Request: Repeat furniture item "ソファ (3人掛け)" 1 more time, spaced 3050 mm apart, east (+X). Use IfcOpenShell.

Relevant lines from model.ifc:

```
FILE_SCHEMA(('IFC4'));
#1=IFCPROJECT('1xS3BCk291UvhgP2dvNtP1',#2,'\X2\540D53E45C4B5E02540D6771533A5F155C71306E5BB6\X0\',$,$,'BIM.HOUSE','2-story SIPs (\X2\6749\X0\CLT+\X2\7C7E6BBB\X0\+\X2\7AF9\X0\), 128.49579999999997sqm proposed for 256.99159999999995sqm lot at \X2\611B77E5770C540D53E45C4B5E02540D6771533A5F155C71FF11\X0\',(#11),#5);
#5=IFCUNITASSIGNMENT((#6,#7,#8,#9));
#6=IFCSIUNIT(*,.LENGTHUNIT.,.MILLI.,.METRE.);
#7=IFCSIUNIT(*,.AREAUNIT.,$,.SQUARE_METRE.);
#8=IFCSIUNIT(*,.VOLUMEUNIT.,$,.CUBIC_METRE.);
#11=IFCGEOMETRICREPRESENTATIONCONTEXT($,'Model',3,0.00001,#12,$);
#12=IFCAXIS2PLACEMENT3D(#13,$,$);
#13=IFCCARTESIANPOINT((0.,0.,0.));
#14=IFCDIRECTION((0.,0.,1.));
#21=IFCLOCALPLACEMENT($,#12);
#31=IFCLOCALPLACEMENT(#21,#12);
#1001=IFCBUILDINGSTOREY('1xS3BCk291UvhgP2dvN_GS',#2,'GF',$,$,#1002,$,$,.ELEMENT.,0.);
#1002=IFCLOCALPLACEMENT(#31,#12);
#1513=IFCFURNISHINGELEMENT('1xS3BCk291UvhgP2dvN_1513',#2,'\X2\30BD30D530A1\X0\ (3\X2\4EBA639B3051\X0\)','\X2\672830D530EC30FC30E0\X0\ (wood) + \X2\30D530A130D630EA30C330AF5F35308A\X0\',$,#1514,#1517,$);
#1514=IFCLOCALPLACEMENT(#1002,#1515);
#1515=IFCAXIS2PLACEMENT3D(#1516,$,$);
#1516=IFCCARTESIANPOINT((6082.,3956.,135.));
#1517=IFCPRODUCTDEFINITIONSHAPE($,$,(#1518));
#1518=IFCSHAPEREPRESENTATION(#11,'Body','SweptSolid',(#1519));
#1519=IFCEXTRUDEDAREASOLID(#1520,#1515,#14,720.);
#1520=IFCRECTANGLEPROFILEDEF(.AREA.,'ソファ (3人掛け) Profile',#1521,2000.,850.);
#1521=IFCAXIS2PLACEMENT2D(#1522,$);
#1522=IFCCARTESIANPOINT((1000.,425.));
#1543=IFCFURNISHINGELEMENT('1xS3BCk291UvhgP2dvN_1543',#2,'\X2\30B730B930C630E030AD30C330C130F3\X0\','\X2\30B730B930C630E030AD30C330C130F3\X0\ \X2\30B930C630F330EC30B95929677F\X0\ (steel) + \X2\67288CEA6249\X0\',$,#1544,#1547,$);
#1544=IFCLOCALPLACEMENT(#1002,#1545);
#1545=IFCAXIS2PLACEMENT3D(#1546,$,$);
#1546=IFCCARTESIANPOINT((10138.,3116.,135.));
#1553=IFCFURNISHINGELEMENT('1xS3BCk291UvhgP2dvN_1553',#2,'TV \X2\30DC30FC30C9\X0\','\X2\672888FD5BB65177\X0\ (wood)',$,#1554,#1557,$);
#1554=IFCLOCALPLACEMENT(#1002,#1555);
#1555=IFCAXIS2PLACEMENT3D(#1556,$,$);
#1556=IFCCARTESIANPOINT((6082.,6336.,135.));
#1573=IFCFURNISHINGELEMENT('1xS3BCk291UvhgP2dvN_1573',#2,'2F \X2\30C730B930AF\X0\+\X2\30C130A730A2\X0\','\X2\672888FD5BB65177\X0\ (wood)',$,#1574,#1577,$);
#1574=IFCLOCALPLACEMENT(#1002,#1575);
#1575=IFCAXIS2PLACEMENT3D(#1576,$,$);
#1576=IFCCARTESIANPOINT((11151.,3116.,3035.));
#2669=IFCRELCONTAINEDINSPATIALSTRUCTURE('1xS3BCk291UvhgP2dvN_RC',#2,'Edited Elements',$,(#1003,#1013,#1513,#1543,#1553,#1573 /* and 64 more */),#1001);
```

```python
import numpy as np
import ifcopenshell
import ifcopenshell.api.geometry
import ifcopenshell.api.root
import ifcopenshell.util.element
import ifcopenshell.util.placement

model = ifcopenshell.open("model.ifc")


def reuse_history(source, copy):
    """copy_class also copies each property set's owner history, people and application; keep the originals."""
    for rel in copy.IsDefinedBy:
        if rel.is_a("IfcRelDefinesByProperties") and (history := rel.RelatingPropertyDefinition.OwnerHistory):
            rel.RelatingPropertyDefinition.OwnerHistory = source.OwnerHistory
            ifcopenshell.util.element.remove_deep2(model, history)


source = model.by_guid("1xS3BCk291UvhgP2dvN_1513")
base = ifcopenshell.util.placement.get_local_placement(source.ObjectPlacement)
step = np.array([1.0, 0.0, 0.0]) * 3050.0

for i in range(1, 2):
    copy = ifcopenshell.api.root.copy_class(model, product=source)
    copy.Representation = ifcopenshell.util.element.copy_deep(
        model, source.Representation, exclude=["IfcGeometricRepresentationContext", "IfcRepresentationMap"]
    )
    reuse_history(source, copy)
    matrix = base.copy()
    matrix[:3, 3] += i * step
    print("added at", matrix[:3, 3].round(3) + 0.0)
    ifcopenshell.api.geometry.edit_object_placement(model, product=copy, matrix=matrix, is_si=False)

model.write("model_rev.ifc")
```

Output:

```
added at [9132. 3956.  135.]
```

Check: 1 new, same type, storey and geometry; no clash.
